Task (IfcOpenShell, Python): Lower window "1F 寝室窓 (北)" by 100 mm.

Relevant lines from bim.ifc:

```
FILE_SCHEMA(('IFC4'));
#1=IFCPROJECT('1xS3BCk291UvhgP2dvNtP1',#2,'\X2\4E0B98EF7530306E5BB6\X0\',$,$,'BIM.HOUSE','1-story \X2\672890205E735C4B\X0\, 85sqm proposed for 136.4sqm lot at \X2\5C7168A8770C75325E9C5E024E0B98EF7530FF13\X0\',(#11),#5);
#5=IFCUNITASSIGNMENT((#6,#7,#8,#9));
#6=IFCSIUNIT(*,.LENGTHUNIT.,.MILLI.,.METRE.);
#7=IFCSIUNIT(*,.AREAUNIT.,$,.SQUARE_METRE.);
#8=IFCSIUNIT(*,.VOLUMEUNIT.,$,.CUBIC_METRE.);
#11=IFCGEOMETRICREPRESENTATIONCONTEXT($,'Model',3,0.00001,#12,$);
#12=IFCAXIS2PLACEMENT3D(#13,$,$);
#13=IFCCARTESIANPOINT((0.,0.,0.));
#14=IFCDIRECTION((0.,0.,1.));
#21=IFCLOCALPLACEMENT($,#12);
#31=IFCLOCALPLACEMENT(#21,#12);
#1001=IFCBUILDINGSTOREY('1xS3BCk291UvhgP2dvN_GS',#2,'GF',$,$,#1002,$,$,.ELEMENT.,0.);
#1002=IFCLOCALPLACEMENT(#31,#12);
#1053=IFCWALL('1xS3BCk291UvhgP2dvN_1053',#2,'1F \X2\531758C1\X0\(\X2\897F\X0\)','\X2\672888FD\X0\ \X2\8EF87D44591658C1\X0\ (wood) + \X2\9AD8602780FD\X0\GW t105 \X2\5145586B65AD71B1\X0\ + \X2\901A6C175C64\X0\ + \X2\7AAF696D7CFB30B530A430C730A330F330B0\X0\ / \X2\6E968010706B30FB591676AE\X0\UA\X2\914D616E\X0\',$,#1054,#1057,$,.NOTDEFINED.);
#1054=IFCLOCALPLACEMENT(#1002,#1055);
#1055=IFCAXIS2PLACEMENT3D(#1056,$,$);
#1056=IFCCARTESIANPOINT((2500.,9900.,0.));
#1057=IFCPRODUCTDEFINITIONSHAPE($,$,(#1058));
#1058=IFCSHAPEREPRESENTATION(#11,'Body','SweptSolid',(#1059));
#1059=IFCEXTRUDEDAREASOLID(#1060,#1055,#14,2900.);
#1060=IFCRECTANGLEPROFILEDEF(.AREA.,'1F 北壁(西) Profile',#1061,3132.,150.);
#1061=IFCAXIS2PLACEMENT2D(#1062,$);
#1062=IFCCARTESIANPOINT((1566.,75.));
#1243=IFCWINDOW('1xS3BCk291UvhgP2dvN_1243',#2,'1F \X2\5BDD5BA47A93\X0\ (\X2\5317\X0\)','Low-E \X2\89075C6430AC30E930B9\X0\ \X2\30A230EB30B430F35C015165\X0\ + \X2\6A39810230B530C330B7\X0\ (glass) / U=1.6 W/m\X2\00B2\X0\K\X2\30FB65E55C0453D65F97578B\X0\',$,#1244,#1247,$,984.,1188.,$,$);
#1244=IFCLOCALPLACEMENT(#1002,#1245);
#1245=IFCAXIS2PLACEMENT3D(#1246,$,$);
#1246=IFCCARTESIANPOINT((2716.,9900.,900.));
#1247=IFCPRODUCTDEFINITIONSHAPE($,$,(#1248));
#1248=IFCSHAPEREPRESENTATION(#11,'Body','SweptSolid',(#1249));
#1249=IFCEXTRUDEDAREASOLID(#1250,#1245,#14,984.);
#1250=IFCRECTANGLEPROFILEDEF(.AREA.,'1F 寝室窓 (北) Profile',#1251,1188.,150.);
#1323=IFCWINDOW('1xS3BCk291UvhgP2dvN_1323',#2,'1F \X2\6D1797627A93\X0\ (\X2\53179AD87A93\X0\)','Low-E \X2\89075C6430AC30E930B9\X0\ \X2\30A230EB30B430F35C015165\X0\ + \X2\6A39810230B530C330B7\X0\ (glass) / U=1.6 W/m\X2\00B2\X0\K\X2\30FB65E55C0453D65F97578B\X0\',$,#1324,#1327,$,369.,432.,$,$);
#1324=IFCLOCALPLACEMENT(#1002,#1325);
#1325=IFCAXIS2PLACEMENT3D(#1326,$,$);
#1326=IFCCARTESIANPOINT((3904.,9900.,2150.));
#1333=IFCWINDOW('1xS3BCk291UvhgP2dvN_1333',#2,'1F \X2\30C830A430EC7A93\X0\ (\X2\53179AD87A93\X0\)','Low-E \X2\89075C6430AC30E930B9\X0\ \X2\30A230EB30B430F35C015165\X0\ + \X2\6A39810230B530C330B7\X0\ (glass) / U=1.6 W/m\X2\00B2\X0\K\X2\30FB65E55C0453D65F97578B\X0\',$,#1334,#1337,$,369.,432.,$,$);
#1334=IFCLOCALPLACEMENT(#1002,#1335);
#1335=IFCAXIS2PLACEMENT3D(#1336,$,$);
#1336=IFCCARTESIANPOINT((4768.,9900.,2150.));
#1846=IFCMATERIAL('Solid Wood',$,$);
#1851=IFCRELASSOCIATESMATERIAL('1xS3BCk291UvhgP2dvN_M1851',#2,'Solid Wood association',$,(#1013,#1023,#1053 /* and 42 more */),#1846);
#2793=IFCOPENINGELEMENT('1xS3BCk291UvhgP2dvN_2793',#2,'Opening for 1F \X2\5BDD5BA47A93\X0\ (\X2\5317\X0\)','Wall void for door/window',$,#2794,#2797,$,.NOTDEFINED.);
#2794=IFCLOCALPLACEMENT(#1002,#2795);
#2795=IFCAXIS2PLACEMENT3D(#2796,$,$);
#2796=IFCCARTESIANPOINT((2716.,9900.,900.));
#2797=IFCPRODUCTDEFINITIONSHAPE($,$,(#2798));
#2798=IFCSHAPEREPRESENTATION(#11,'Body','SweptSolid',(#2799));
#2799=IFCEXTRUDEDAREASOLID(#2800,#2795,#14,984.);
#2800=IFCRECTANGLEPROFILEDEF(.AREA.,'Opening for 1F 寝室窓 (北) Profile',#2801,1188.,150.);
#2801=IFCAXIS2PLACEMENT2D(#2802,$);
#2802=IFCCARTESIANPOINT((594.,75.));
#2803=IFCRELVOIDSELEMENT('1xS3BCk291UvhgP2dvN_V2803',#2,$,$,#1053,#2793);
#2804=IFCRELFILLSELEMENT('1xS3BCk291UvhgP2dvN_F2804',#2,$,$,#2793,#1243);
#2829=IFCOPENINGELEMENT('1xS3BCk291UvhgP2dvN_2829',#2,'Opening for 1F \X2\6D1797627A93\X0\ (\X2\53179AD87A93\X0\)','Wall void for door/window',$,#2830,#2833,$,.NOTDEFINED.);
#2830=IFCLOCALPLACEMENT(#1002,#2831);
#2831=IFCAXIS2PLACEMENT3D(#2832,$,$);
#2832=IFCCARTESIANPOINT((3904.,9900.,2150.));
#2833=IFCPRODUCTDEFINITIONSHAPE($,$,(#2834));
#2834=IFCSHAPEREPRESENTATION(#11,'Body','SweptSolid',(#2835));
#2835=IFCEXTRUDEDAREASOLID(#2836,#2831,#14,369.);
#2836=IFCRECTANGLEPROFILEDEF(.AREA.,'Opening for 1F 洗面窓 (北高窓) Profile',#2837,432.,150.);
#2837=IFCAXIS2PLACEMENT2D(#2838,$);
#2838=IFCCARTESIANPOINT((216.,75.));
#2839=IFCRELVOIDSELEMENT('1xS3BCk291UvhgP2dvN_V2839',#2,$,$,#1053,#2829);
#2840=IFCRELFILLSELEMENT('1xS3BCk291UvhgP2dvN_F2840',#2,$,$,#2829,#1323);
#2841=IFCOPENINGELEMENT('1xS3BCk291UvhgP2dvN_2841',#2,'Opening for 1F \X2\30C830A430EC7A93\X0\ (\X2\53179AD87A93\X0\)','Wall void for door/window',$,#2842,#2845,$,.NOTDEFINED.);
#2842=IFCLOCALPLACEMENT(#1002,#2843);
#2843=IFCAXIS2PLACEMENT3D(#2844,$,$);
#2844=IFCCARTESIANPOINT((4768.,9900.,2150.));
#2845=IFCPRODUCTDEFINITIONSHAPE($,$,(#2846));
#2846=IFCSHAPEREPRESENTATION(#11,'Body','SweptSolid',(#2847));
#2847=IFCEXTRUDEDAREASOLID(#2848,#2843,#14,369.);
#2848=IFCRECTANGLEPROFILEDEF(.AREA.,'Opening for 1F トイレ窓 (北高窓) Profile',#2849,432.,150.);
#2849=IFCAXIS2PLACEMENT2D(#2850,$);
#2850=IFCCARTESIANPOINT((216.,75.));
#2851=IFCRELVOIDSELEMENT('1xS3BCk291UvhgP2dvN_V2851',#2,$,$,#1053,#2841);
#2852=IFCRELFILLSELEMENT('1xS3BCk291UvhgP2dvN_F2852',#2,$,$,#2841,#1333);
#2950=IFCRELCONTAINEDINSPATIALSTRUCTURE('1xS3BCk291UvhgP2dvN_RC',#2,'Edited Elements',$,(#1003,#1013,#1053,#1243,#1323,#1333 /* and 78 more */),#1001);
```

```python
import numpy as np
import ifcopenshell
import ifcopenshell.api.geometry
import ifcopenshell.util.placement
import ifcopenshell.util.unit

model = ifcopenshell.open("bim.ifc")
unit_scale = ifcopenshell.util.unit.calculate_unit_scale(model)

window = model.by_guid("1xS3BCk291UvhgP2dvN_1243")
opening = window.FillsVoids[0].RelatingOpeningElement
dz = -0.1 / unit_scale

shift = np.array([0.0, 0.0, dz])
# The window is not placed relative to its opening, so move both.
for product in (opening, window):
    matrix = ifcopenshell.util.placement.get_local_placement(product.ObjectPlacement)
    matrix[:3, 3] += shift
    ifcopenshell.api.geometry.edit_object_placement(model, product=product, matrix=matrix, is_si=False)

print(f"moved by {dz * unit_scale:+.3f} m")

model.write("bim_rev.ifc")
```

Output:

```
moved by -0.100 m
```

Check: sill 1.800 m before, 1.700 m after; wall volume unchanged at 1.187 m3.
